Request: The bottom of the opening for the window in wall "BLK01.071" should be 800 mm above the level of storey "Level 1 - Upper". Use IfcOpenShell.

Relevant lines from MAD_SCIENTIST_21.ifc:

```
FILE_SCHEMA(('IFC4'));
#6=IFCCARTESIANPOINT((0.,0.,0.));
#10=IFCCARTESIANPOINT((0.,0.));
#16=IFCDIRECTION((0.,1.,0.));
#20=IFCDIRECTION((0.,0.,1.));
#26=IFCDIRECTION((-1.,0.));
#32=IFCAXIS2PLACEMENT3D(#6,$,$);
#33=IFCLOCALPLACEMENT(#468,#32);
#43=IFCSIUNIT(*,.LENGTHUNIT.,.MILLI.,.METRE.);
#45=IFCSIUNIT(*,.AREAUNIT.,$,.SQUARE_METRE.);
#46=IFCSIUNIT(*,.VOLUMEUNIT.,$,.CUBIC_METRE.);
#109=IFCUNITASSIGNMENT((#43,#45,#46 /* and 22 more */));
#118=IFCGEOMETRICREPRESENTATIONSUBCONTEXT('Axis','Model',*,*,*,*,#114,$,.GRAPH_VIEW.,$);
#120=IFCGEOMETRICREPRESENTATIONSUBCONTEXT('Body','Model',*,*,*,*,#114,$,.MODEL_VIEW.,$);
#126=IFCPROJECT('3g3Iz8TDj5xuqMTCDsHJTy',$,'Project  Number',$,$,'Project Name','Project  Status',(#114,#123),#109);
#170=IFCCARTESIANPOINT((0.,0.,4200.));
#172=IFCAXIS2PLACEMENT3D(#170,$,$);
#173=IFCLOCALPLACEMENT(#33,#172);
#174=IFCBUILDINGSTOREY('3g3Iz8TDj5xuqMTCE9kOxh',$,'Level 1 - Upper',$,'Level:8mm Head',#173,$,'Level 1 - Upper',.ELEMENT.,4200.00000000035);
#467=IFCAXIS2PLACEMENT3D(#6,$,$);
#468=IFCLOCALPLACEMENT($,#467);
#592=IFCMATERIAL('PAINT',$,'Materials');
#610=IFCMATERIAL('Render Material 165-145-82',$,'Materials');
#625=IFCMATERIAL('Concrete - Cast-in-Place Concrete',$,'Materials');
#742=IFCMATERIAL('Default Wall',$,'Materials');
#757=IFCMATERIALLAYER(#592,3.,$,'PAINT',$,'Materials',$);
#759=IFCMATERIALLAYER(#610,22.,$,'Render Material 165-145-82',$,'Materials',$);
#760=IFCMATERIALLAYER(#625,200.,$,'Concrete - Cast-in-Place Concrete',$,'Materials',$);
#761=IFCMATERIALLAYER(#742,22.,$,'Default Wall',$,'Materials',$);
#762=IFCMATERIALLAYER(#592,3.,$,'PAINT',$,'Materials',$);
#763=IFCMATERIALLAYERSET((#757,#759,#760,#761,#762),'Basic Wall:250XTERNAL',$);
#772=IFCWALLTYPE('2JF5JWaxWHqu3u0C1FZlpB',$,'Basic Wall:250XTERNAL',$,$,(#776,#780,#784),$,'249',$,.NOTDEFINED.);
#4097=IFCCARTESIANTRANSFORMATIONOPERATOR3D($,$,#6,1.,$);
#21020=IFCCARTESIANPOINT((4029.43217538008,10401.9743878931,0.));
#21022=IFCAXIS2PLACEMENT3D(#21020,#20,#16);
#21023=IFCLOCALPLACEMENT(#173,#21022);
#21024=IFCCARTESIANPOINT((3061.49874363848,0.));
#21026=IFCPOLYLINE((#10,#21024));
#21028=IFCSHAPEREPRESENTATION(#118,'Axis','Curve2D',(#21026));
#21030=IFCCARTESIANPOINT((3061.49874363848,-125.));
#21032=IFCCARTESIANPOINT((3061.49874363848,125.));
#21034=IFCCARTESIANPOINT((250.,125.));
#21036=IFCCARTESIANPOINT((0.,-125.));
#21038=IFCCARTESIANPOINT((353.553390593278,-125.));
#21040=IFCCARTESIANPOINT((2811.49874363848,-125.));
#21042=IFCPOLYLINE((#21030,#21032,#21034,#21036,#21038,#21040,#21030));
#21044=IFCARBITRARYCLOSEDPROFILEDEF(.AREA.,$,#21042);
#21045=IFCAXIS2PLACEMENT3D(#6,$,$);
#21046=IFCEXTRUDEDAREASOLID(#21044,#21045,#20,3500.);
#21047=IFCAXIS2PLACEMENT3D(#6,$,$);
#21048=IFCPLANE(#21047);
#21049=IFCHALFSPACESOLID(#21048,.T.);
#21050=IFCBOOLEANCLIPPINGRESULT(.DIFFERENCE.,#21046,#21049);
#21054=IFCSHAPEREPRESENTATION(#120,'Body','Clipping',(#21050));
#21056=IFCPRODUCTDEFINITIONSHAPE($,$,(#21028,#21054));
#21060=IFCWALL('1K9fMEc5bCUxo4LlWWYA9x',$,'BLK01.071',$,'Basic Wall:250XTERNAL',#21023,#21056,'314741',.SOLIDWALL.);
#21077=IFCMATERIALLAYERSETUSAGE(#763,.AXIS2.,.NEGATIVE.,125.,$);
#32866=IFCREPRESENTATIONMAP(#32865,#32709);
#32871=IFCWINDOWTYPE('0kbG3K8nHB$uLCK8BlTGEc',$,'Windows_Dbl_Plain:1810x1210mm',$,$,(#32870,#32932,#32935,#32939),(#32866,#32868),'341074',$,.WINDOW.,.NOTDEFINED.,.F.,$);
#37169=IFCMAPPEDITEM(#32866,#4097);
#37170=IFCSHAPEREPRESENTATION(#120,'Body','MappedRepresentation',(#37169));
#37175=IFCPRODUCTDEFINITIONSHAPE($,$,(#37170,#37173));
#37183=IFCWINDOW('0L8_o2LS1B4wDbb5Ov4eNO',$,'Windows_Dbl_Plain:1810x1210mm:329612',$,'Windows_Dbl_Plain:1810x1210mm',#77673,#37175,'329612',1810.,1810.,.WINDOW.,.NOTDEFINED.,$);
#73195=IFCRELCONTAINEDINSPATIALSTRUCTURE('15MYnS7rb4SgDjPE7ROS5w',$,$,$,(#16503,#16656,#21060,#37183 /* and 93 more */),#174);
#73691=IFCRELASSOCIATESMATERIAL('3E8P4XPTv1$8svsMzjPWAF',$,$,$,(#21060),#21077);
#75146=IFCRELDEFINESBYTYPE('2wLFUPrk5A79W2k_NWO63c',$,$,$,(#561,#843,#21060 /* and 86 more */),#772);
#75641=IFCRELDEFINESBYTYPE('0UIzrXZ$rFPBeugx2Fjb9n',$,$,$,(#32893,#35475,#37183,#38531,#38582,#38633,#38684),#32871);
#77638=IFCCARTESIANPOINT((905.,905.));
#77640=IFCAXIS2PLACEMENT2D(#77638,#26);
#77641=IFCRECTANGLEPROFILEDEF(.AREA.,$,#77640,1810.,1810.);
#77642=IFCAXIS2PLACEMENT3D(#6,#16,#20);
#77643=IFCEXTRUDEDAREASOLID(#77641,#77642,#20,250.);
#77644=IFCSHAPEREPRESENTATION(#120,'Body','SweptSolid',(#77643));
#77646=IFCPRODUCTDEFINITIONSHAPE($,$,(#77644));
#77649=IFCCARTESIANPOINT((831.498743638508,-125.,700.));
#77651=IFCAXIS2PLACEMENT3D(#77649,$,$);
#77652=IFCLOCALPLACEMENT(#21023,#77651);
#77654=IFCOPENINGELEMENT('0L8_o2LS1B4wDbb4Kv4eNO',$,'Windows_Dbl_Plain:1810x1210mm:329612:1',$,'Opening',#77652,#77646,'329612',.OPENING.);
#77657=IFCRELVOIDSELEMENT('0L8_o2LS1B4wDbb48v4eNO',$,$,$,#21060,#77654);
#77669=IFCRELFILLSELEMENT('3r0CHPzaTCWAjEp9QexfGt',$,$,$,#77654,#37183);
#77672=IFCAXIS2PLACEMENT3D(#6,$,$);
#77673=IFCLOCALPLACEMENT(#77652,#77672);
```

```python
import numpy as np
import ifcopenshell
import ifcopenshell.api.geometry
import ifcopenshell.geom
import ifcopenshell.util.element
import ifcopenshell.util.placement
import ifcopenshell.util.shape
import ifcopenshell.util.unit

model = ifcopenshell.open("MAD_SCIENTIST_21.ifc")
unit_scale = ifcopenshell.util.unit.calculate_unit_scale(model)

window = model.by_guid("0L8_o2LS1B4wDbb5Ov4eNO")
opening = window.FillsVoids[0].RelatingOpeningElement
storey = ifcopenshell.util.element.get_container(window, ifc_class="IfcBuildingStorey")
level = ifcopenshell.util.placement.get_local_placement(storey.ObjectPlacement)[2, 3]

# The opening's origin need not be at the sill, so measure its lowest point.
shape = ifcopenshell.geom.create_shape(ifcopenshell.geom.settings(), opening)
bottom = ifcopenshell.util.shape.get_shape_bottom_elevation(shape, shape.geometry) / unit_scale
dz = level + 800.0 - bottom

shift = np.array([0.0, 0.0, dz])
# The window is placed relative to its opening, so it follows when the opening moves.
matrix = ifcopenshell.util.placement.get_local_placement(opening.ObjectPlacement)
matrix[:3, 3] += shift
ifcopenshell.api.geometry.edit_object_placement(
    model, product=opening, matrix=matrix, is_si=False, should_transform_children=True
)

print(f"moved by {dz * unit_scale:+.3f} m")

model.write("MAD_SCIENTIST_21_rev.ifc")
```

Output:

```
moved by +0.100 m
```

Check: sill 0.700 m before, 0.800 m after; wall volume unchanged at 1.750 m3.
